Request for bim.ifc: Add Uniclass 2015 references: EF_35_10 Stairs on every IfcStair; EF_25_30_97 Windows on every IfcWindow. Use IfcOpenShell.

First a look at what the model holds.

```python
import ifcopenshell

model = ifcopenshell.open("bim.ifc")
print(model.schema)
print("classifications:", [c.Name for c in model.by_type("IfcClassification")])
for ifc_class in ("IfcDoor", "IfcRoof", "IfcStair", "IfcWall", "IfcWindow"):
    print(ifc_class, len(model.by_type(ifc_class)))
```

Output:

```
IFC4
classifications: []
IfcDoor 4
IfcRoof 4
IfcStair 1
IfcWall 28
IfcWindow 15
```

```python
import ifcopenshell
import ifcopenshell.api.classification

model = ifcopenshell.open("bim.ifc")

system = ifcopenshell.api.classification.add_classification(model, classification="Uniclass 2015")

codes = {
    "IfcStair": ("EF_35_10", "Stairs"),
    "IfcWindow": ("EF_25_30_97", "Windows"),
}
for ifc_class, (code, name) in codes.items():
    products = model.by_type(ifc_class)
    ifcopenshell.api.classification.add_reference(
        model, products=products, classification=system, identification=code, name=name
    )
    print(code, len(products))

model.write("bim_rev.ifc")
```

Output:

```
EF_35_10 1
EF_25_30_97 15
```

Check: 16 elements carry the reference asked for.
